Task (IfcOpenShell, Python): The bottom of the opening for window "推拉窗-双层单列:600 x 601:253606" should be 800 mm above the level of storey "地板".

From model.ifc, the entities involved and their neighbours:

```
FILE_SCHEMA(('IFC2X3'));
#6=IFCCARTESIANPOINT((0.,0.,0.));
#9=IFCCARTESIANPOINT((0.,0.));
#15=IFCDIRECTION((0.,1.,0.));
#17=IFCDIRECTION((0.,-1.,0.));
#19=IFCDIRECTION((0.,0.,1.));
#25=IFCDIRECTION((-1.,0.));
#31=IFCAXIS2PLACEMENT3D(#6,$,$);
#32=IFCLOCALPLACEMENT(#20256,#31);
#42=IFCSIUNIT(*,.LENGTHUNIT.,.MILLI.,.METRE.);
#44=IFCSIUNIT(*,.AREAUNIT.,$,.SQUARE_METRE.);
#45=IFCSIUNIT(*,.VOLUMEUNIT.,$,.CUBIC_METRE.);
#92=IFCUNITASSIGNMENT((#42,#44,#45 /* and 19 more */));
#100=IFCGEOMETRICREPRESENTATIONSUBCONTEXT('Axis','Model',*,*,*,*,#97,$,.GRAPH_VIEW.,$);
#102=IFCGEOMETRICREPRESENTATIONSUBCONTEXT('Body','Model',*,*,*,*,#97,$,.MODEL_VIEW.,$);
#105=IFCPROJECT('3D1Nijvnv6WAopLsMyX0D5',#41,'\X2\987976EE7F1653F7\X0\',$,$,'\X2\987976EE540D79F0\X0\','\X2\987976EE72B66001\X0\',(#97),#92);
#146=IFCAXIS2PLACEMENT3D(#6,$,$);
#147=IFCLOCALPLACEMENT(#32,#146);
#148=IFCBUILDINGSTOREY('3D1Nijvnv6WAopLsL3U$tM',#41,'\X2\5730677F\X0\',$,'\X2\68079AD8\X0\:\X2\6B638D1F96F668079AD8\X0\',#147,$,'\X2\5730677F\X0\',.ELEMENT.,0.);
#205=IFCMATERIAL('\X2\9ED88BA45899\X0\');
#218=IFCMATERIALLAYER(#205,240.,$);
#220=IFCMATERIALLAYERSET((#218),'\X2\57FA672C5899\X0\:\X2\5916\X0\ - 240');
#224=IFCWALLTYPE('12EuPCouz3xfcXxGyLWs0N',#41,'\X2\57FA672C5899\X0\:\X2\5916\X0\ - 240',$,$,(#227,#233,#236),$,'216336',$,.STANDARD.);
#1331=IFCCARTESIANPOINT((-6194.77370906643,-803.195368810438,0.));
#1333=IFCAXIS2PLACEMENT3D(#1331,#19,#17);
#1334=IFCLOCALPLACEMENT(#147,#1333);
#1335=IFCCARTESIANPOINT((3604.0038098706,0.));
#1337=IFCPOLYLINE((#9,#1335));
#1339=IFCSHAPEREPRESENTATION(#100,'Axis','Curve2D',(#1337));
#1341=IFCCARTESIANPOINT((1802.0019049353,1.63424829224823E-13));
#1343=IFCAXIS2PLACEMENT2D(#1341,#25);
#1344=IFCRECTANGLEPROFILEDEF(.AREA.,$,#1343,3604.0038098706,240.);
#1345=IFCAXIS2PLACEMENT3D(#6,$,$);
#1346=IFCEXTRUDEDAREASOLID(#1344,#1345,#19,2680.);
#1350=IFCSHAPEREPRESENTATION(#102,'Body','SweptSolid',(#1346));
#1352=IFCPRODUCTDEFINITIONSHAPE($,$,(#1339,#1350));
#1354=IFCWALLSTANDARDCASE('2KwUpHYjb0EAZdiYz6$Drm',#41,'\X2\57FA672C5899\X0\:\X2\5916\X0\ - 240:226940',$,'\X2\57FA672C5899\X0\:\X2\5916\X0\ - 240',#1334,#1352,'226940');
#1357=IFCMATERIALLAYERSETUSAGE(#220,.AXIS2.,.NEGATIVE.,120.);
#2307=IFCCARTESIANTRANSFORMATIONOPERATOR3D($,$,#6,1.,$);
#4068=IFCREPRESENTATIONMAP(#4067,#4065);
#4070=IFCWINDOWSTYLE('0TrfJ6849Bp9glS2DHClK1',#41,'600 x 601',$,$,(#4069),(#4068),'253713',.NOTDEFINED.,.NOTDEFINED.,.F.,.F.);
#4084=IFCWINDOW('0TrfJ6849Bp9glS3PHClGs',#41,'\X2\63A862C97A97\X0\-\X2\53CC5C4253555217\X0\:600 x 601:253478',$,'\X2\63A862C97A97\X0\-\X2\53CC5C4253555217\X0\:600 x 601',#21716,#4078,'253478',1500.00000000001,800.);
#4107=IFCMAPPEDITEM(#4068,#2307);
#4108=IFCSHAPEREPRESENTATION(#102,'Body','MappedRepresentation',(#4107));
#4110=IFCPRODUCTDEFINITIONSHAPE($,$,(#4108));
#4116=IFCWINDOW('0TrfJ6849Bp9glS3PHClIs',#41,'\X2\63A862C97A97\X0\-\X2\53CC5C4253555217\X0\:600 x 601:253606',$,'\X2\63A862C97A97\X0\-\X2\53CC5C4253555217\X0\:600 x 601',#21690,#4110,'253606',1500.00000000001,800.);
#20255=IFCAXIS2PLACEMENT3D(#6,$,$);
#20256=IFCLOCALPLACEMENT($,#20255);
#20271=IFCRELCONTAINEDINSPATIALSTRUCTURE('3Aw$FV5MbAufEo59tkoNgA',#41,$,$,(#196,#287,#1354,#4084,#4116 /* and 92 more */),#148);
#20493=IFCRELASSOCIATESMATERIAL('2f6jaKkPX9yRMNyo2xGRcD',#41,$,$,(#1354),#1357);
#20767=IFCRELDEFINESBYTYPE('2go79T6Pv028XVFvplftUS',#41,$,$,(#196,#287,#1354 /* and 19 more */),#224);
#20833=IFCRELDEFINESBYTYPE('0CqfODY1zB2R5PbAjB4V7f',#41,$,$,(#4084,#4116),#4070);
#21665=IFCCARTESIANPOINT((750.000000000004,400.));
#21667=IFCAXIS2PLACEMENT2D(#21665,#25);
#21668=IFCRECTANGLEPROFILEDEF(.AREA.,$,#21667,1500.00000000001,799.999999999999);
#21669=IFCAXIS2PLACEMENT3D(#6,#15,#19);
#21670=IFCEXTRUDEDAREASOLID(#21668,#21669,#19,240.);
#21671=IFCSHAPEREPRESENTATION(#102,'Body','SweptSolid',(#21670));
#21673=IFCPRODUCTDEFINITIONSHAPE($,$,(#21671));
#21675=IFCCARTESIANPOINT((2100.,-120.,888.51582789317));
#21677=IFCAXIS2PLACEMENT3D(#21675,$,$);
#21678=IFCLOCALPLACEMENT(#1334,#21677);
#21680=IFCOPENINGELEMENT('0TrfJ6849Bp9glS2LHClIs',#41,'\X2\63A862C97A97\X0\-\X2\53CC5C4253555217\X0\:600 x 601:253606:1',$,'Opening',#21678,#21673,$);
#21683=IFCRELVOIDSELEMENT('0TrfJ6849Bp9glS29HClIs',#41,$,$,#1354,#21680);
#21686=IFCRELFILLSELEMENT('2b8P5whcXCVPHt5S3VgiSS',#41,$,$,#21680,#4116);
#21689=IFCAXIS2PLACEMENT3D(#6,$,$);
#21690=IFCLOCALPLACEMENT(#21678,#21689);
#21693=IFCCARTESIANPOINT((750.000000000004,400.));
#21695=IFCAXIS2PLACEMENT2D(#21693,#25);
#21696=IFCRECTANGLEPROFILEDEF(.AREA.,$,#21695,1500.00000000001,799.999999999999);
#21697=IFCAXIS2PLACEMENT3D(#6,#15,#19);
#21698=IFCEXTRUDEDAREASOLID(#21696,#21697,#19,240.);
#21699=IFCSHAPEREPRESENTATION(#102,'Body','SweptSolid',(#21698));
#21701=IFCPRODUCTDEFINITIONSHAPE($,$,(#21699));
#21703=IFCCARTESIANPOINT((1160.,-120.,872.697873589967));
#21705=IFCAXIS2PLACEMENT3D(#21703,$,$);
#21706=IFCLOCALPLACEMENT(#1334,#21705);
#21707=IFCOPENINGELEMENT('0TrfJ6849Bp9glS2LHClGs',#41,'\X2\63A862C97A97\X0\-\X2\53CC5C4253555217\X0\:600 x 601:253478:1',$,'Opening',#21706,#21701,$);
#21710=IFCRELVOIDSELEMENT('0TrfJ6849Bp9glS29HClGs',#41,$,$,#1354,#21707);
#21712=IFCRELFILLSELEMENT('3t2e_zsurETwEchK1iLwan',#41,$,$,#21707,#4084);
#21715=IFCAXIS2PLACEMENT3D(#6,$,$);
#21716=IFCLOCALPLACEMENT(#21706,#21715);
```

```python
import numpy as np
import ifcopenshell
import ifcopenshell.api.geometry
import ifcopenshell.geom
import ifcopenshell.util.element
import ifcopenshell.util.placement
import ifcopenshell.util.shape
import ifcopenshell.util.unit

model = ifcopenshell.open("model.ifc")
unit_scale = ifcopenshell.util.unit.calculate_unit_scale(model)

window = model.by_guid("0TrfJ6849Bp9glS3PHClIs")
opening = window.FillsVoids[0].RelatingOpeningElement
storey = ifcopenshell.util.element.get_container(window, ifc_class="IfcBuildingStorey")
level = ifcopenshell.util.placement.get_local_placement(storey.ObjectPlacement)[2, 3]

# The opening's origin need not be at the sill, so measure its lowest point.
shape = ifcopenshell.geom.create_shape(ifcopenshell.geom.settings(), opening)
bottom = ifcopenshell.util.shape.get_shape_bottom_elevation(shape, shape.geometry) / unit_scale
dz = level + 800.0 - bottom

shift = np.array([0.0, 0.0, dz])
# The window is placed relative to its opening, so it follows when the opening moves.
matrix = ifcopenshell.util.placement.get_local_placement(opening.ObjectPlacement)
matrix[:3, 3] += shift
ifcopenshell.api.geometry.edit_object_placement(
    model, product=opening, matrix=matrix, is_si=False, should_transform_children=True
)

print(f"moved by {dz * unit_scale:+.3f} m")

model.write("model_edited.ifc")
```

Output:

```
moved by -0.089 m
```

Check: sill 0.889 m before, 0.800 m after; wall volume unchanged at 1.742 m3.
